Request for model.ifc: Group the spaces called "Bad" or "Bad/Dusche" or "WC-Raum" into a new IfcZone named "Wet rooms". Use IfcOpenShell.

First a look at what the model holds.

```python
import ifcopenshell

model = ifcopenshell.open("model.ifc")
print(model.schema)
seen = {}
for space in model.by_type("IfcSpace"):
    seen[space.Name] = seen.get(space.Name, 0) + 1
for name, count in sorted(seen.items(), key=str):
    print(count, "x", name)
print("zones:", [z.Name for z in model.by_type("IfcZone")][:20])
```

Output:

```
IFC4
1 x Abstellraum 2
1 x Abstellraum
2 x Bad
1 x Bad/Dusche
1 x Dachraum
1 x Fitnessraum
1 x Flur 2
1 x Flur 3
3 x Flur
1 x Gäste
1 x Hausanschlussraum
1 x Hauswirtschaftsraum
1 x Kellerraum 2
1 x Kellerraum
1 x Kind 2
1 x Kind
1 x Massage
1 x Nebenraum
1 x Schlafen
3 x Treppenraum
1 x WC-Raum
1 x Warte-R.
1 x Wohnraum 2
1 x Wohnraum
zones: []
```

```python
import ifcopenshell
import ifcopenshell.api.group
import ifcopenshell.api.root

model = ifcopenshell.open("model.ifc")

names = {"Bad", "Bad/Dusche", "WC-Raum"}
spaces = [s for s in model.by_type("IfcSpace") if s.Name in names]

zone = ifcopenshell.api.root.create_entity(model, ifc_class="IfcZone", name="Wet rooms")
ifcopenshell.api.group.assign_group(model, products=spaces, group=zone)
print(len(spaces), "spaces in", zone.Name)

model.write("model_v2.ifc")
```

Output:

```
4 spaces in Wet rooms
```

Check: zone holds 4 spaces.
